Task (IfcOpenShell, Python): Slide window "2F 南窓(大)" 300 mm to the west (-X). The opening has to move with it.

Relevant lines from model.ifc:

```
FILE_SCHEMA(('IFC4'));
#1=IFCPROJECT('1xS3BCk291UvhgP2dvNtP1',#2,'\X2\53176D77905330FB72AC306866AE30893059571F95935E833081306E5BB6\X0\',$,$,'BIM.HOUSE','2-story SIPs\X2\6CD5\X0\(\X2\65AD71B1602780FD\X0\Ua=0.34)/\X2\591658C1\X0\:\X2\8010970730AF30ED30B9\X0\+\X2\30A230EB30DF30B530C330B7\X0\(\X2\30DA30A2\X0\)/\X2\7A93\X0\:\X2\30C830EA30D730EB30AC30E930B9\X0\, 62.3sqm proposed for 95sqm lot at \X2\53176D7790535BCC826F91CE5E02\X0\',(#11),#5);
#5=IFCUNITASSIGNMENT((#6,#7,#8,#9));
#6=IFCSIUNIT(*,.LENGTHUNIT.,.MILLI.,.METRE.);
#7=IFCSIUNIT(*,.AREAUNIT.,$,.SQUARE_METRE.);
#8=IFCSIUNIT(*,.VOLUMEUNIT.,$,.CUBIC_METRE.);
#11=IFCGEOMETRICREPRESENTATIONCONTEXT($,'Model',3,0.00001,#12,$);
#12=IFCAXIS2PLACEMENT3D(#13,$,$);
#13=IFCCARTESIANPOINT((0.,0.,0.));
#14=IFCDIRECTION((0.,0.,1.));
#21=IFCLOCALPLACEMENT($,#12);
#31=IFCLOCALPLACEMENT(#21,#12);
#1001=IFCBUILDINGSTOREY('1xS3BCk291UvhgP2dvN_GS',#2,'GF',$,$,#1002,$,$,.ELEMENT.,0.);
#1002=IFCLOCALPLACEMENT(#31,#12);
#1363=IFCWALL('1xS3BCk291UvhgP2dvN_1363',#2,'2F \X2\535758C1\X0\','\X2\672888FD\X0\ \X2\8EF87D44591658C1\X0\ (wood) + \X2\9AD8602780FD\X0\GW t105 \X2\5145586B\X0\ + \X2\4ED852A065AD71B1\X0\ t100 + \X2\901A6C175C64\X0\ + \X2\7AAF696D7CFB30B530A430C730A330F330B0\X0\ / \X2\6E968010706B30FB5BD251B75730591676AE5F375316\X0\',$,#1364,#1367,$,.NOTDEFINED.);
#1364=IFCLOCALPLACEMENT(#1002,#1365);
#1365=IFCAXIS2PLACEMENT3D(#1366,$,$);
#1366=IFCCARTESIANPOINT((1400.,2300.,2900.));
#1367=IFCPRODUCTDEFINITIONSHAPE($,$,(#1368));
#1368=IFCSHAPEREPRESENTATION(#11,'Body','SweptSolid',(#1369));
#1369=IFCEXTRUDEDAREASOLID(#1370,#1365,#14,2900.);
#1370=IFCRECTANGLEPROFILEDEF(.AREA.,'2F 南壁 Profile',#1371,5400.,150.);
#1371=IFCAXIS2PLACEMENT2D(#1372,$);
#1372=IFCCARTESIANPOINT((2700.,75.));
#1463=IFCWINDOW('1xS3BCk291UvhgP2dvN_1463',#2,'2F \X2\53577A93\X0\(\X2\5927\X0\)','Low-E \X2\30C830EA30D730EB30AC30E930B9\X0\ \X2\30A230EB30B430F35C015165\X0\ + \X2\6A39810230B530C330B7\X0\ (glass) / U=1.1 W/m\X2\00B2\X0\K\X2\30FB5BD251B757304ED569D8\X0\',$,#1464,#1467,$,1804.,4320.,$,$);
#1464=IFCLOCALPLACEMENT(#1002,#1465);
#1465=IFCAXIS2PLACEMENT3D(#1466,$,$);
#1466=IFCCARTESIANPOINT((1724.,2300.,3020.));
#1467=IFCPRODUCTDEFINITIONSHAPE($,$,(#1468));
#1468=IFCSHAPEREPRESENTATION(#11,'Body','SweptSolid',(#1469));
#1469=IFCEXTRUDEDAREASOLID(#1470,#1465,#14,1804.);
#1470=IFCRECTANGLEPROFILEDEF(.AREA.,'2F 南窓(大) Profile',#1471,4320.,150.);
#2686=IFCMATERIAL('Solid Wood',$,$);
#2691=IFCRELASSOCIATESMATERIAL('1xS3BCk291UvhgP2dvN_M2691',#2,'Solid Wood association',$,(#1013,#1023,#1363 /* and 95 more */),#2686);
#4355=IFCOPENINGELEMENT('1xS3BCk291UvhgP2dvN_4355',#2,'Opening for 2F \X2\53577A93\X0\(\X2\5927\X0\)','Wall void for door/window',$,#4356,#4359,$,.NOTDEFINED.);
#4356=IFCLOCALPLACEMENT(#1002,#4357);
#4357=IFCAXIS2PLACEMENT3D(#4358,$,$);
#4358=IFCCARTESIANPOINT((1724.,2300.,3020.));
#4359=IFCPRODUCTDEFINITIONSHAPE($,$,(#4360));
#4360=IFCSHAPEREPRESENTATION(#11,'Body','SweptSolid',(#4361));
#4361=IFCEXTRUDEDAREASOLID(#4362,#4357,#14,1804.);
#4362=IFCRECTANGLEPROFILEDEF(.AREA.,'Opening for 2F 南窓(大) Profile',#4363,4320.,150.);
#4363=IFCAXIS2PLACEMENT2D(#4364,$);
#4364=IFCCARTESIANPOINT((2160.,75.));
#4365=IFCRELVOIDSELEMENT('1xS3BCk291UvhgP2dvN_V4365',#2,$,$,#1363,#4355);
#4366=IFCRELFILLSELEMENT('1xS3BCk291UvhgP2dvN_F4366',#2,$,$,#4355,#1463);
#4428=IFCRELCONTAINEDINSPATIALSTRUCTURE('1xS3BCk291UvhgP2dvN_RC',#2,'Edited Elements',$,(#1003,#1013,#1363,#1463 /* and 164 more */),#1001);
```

```python
import ifcopenshell
import ifcopenshell.api.geometry
import ifcopenshell.util.placement
import ifcopenshell.util.unit

model = ifcopenshell.open("model.ifc")
unit_scale = ifcopenshell.util.unit.calculate_unit_scale(model)

window = model.by_guid("1xS3BCk291UvhgP2dvN_1463")
opening = window.FillsVoids[0].RelatingOpeningElement
wall = opening.VoidsElements[0].RelatingBuildingElement

wall_matrix = ifcopenshell.util.placement.get_local_placement(wall.ObjectPlacement)
shift = wall_matrix[:3, 0] * -0.3 / unit_scale
before = ifcopenshell.util.placement.get_local_placement(window.ObjectPlacement)[:3, 3].copy()

# The window is not placed relative to its opening, so move both.
for product in (opening, window):
    matrix = ifcopenshell.util.placement.get_local_placement(product.ObjectPlacement)
    matrix[:3, 3] += shift
    ifcopenshell.api.geometry.edit_object_placement(model, product=product, matrix=matrix, is_si=False)

after = ifcopenshell.util.placement.get_local_placement(window.ObjectPlacement)[:3, 3]
print("window moved by", (after - before).round(3) + 0.0)

model.write("model_v2.ifc")
```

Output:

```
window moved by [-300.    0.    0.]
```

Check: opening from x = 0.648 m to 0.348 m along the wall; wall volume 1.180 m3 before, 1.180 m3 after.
